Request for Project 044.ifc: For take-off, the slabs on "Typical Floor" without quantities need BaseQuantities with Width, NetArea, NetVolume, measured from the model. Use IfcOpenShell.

First a look at what the model holds.

```python
import ifcopenshell
import ifcopenshell.util.element
import ifcopenshell.util.unit

model = ifcopenshell.open("Project 044.ifc")
print(model.schema)
for unit_type in ("LENGTHUNIT", "AREAUNIT", "VOLUMEUNIT"):
    print(unit_type, ifcopenshell.util.unit.calculate_unit_scale(model, unit_type))
storey = next(s for s in model.by_type("IfcBuildingStorey") if s.Name == "Typical Floor")
slabs = [e for e in ifcopenshell.util.element.get_decomposition(storey) if e.is_a("IfcSlab")]
for e in sorted(slabs, key=lambda e: e.id()):
    print(e.id(), e.is_a(), e.Name, list(ifcopenshell.util.element.get_psets(e, qtos_only=True)), sep=" | ")
```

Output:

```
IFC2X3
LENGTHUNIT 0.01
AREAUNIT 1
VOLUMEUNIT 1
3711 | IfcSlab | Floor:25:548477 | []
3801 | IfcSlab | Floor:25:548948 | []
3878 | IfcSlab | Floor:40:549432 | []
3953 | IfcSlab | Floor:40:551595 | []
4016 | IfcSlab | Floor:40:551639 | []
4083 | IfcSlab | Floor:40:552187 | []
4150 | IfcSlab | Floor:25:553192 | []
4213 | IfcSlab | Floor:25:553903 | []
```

```python
import ifcopenshell
import ifcopenshell.api.pset
import ifcopenshell.geom
import ifcopenshell.util.element
import ifcopenshell.util.shape
import ifcopenshell.util.unit

model = ifcopenshell.open("Project 044.ifc")
unit_scale = ifcopenshell.util.unit.calculate_unit_scale(model)
area_scale = ifcopenshell.util.unit.calculate_unit_scale(model, "AREAUNIT")
volume_scale = ifcopenshell.util.unit.calculate_unit_scale(model, "VOLUMEUNIT")
settings = ifcopenshell.geom.settings()

storey = next(s for s in model.by_type("IfcBuildingStorey") if s.Name == "Typical Floor")
slabs = [e for e in ifcopenshell.util.element.get_decomposition(storey) if e.is_a("IfcSlab")]

for e in sorted(slabs, key=lambda e: e.id()):
    if ifcopenshell.util.element.get_psets(e, qtos_only=True, should_inherit=False):
        continue
    # Geometry comes back in metres, in the element's own axes.
    shape = ifcopenshell.geom.create_shape(settings, e)
    values = {
        "Width": ifcopenshell.util.shape.get_z(shape.geometry) / unit_scale,
        "NetArea": ifcopenshell.util.shape.get_footprint_area(shape.geometry) / area_scale,
        "NetVolume": ifcopenshell.util.shape.get_volume(shape.geometry) / volume_scale,
    }
    qto = ifcopenshell.api.pset.add_qto(model, product=e, name="BaseQuantities")
    ifcopenshell.api.pset.edit_qto(model, qto=qto, properties=values)
    print(e.id(), {k: round(v, 3) for k, v in values.items()})

model.write("Project 044-out.ifc")
```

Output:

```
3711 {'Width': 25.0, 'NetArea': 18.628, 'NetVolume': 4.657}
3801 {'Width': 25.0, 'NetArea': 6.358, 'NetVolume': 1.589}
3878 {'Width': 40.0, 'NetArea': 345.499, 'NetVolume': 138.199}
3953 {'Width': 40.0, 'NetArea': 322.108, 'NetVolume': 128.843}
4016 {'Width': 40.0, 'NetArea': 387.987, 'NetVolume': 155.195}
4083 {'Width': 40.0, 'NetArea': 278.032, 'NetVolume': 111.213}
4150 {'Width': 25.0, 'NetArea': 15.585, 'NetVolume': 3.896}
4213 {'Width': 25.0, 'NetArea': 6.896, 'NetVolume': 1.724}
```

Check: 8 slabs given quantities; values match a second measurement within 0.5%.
